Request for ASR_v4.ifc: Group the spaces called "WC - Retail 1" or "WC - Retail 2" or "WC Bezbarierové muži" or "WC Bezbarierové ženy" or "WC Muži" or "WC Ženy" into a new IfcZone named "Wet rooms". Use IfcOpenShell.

First a look at what the model holds.

```python
import ifcopenshell

model = ifcopenshell.open("ASR_v4.ifc")
print(model.schema)
seen = {}
for space in model.by_type("IfcSpace"):
    seen[space.LongName] = seen.get(space.LongName, 0) + 1
for name, count in sorted(seen.items(), key=str):
    print(count, "x", name)
print("zones:", [z.Name for z in model.by_type("IfcZone")][:20])
```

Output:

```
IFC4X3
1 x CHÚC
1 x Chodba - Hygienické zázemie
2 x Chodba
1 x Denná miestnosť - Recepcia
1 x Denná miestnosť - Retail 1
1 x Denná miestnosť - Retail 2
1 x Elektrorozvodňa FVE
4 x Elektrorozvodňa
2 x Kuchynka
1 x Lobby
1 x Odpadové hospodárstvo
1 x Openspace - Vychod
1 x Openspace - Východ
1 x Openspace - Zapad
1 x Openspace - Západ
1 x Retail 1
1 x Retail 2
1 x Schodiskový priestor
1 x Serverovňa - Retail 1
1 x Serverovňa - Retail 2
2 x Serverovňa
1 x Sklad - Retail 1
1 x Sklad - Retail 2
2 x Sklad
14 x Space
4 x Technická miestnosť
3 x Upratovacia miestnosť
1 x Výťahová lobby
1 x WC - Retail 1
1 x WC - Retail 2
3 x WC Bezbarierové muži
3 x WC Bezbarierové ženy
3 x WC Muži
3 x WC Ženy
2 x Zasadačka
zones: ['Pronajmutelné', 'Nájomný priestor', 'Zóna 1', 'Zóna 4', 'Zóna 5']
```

```python
import ifcopenshell
import ifcopenshell.api.group
import ifcopenshell.api.root

model = ifcopenshell.open("ASR_v4.ifc")

names = {"WC - Retail 1", "WC - Retail 2", "WC Bezbarierové muži", "WC Bezbarierové ženy", "WC Muži", "WC Ženy"}
spaces = [s for s in model.by_type("IfcSpace") if s.LongName in names]

zone = ifcopenshell.api.root.create_entity(model, ifc_class="IfcZone", name="Wet rooms")
ifcopenshell.api.group.assign_group(model, products=spaces, group=zone)
print(len(spaces), "spaces in", zone.Name)

model.write("ASR_v4_edited.ifc")
```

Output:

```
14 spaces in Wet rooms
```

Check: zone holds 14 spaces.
